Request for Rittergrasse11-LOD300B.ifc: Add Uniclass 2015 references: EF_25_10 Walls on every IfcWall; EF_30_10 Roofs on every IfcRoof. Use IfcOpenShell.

First a look at what the model holds.

```python
import ifcopenshell

model = ifcopenshell.open("Rittergrasse11-LOD300B.ifc")
print(model.schema)
print("classifications:", [c.Name for c in model.by_type("IfcClassification")])
for ifc_class in ("IfcDoor", "IfcRoof", "IfcStair", "IfcWall", "IfcWindow"):
    print(ifc_class, len(model.by_type(ifc_class)))
```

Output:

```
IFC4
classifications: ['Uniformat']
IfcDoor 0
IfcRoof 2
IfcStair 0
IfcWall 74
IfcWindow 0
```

```python
import ifcopenshell
import ifcopenshell.api.classification

model = ifcopenshell.open("Rittergrasse11-LOD300B.ifc")

system = ifcopenshell.api.classification.add_classification(model, classification="Uniclass 2015")

codes = {
    "IfcWall": ("EF_25_10", "Walls"),
    "IfcRoof": ("EF_30_10", "Roofs"),
}
for ifc_class, (code, name) in codes.items():
    products = model.by_type(ifc_class)
    ifcopenshell.api.classification.add_reference(
        model, products=products, classification=system, identification=code, name=name
    )
    print(code, len(products))

model.write("Rittergrasse11-LOD300B-out.ifc")
```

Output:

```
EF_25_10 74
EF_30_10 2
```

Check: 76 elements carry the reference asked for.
